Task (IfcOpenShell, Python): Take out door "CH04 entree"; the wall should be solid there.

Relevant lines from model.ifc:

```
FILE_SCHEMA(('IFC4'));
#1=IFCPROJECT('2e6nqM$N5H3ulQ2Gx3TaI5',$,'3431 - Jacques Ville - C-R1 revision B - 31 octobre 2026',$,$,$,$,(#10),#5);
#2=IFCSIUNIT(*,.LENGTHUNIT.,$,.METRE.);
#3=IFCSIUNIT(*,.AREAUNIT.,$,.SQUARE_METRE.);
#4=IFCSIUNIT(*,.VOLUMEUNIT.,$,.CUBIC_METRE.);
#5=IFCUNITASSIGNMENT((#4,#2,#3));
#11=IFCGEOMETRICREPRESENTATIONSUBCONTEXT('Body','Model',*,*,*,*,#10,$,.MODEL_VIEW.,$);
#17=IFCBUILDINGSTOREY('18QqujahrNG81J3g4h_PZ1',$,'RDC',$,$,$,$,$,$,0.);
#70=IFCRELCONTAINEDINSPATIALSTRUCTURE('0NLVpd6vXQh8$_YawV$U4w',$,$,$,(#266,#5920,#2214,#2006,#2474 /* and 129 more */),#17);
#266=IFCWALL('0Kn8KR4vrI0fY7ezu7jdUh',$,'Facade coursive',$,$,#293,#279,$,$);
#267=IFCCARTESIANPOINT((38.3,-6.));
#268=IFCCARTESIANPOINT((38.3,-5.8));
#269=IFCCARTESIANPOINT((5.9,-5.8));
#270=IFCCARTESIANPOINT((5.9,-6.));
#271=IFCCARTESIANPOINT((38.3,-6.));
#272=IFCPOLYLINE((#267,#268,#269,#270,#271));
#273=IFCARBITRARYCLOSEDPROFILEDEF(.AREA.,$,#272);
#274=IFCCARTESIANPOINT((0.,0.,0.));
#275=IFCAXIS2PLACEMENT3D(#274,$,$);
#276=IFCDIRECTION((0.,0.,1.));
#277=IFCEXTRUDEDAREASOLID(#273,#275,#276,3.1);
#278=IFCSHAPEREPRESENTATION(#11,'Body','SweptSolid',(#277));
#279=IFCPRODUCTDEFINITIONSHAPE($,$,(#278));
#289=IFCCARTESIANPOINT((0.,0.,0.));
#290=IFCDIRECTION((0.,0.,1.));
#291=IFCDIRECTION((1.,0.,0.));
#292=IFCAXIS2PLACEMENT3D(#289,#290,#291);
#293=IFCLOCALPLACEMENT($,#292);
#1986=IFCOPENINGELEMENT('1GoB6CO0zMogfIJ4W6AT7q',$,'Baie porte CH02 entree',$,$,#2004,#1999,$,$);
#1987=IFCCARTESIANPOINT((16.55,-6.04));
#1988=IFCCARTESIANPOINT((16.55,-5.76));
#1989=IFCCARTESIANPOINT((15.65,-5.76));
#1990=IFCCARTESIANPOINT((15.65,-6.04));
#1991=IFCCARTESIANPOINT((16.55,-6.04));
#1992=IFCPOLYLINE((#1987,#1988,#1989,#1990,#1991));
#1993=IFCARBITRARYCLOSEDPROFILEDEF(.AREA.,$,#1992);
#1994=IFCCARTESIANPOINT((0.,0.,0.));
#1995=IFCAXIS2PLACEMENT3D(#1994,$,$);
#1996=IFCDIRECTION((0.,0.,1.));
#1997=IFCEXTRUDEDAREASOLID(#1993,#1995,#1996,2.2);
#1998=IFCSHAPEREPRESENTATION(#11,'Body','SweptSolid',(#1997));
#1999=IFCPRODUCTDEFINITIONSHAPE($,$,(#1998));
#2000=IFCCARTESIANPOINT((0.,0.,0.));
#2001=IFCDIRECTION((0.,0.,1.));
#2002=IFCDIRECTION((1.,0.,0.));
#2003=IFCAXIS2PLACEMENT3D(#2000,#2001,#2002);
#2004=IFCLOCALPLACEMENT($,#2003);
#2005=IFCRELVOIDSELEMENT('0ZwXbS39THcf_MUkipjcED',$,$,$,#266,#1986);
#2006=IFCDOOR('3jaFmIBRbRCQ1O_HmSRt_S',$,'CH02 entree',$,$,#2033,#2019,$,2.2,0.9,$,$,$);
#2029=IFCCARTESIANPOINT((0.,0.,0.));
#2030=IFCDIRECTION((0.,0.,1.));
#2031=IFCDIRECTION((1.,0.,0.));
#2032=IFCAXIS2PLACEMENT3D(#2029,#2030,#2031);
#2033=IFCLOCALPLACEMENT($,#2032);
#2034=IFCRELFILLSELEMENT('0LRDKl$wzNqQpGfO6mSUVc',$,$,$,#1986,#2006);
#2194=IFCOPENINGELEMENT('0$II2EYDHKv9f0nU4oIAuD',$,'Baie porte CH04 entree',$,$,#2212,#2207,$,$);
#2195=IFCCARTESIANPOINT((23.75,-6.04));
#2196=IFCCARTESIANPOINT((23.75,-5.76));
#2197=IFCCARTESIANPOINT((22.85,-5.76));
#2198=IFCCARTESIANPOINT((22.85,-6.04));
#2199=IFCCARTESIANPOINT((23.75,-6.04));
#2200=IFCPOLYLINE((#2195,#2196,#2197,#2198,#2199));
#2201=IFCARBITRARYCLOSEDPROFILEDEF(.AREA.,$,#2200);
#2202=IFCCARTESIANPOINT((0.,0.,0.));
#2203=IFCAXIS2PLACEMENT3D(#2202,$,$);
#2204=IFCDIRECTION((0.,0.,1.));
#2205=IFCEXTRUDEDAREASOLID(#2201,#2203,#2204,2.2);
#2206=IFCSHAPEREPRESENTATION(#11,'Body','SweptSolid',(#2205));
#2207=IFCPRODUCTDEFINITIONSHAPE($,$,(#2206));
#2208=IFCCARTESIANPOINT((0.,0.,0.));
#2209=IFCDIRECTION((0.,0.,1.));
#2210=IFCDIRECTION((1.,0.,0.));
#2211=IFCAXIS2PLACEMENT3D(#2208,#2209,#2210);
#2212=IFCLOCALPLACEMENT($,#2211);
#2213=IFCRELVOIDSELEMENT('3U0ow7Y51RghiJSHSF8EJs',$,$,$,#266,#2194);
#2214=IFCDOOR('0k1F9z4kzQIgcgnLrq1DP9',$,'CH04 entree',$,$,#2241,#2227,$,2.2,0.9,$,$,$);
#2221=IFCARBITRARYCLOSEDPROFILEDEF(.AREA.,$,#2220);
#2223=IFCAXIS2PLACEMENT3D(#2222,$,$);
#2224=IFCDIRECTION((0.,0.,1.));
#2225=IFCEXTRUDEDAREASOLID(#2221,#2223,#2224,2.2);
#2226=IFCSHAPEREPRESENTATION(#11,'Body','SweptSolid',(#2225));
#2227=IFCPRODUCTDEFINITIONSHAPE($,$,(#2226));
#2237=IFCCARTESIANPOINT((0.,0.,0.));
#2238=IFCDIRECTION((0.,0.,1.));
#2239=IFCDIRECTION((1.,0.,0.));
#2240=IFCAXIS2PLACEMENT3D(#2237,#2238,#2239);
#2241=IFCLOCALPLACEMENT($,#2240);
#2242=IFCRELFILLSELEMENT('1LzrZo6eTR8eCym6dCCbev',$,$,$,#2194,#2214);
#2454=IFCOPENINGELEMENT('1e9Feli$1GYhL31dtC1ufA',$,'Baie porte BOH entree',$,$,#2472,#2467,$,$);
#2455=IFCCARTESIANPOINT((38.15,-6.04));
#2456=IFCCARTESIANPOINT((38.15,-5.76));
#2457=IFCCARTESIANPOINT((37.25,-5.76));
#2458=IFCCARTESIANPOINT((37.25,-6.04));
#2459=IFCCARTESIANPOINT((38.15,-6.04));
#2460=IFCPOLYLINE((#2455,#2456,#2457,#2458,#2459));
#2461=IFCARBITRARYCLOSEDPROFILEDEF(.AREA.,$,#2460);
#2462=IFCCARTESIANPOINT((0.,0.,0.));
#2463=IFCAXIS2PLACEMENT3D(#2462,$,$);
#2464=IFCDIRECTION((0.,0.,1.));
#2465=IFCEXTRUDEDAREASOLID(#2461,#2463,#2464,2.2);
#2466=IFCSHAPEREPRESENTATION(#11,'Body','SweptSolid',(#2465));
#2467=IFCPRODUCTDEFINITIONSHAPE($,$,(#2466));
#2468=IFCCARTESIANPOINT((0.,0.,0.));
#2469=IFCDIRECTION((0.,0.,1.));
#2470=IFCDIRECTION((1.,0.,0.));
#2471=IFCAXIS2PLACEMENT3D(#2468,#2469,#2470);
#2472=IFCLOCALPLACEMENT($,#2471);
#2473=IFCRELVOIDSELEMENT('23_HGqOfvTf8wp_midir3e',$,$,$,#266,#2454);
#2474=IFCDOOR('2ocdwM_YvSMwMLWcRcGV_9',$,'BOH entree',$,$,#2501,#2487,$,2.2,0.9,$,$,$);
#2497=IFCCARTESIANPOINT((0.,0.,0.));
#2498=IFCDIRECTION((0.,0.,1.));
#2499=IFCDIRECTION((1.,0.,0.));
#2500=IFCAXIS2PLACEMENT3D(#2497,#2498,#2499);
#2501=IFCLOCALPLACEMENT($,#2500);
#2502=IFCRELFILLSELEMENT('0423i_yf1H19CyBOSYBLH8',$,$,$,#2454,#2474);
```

```python
import ifcopenshell
import ifcopenshell.api.feature
import ifcopenshell.api.root
import ifcopenshell.geom
import ifcopenshell.util.shape

model = ifcopenshell.open("model.ifc")
settings = ifcopenshell.geom.settings()


def volume(element):
    """Net volume in cubic metres, openings subtracted."""
    shape = ifcopenshell.geom.create_shape(settings, element)
    return ifcopenshell.util.shape.get_volume(shape.geometry)


door = model.by_id(2214)
opening = door.FillsVoids[0].RelatingOpeningElement
wall = opening.VoidsElements[0].RelatingBuildingElement
before = volume(wall)

ifcopenshell.api.root.remove_product(model, product=door)
ifcopenshell.api.feature.remove_feature(model, feature=opening)

after = volume(wall)

print(f"wall volume {before:.3f} -> {after:.3f} m3")

model.write("model_updated.ifc")
```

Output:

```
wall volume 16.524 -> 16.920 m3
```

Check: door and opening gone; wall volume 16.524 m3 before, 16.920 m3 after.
